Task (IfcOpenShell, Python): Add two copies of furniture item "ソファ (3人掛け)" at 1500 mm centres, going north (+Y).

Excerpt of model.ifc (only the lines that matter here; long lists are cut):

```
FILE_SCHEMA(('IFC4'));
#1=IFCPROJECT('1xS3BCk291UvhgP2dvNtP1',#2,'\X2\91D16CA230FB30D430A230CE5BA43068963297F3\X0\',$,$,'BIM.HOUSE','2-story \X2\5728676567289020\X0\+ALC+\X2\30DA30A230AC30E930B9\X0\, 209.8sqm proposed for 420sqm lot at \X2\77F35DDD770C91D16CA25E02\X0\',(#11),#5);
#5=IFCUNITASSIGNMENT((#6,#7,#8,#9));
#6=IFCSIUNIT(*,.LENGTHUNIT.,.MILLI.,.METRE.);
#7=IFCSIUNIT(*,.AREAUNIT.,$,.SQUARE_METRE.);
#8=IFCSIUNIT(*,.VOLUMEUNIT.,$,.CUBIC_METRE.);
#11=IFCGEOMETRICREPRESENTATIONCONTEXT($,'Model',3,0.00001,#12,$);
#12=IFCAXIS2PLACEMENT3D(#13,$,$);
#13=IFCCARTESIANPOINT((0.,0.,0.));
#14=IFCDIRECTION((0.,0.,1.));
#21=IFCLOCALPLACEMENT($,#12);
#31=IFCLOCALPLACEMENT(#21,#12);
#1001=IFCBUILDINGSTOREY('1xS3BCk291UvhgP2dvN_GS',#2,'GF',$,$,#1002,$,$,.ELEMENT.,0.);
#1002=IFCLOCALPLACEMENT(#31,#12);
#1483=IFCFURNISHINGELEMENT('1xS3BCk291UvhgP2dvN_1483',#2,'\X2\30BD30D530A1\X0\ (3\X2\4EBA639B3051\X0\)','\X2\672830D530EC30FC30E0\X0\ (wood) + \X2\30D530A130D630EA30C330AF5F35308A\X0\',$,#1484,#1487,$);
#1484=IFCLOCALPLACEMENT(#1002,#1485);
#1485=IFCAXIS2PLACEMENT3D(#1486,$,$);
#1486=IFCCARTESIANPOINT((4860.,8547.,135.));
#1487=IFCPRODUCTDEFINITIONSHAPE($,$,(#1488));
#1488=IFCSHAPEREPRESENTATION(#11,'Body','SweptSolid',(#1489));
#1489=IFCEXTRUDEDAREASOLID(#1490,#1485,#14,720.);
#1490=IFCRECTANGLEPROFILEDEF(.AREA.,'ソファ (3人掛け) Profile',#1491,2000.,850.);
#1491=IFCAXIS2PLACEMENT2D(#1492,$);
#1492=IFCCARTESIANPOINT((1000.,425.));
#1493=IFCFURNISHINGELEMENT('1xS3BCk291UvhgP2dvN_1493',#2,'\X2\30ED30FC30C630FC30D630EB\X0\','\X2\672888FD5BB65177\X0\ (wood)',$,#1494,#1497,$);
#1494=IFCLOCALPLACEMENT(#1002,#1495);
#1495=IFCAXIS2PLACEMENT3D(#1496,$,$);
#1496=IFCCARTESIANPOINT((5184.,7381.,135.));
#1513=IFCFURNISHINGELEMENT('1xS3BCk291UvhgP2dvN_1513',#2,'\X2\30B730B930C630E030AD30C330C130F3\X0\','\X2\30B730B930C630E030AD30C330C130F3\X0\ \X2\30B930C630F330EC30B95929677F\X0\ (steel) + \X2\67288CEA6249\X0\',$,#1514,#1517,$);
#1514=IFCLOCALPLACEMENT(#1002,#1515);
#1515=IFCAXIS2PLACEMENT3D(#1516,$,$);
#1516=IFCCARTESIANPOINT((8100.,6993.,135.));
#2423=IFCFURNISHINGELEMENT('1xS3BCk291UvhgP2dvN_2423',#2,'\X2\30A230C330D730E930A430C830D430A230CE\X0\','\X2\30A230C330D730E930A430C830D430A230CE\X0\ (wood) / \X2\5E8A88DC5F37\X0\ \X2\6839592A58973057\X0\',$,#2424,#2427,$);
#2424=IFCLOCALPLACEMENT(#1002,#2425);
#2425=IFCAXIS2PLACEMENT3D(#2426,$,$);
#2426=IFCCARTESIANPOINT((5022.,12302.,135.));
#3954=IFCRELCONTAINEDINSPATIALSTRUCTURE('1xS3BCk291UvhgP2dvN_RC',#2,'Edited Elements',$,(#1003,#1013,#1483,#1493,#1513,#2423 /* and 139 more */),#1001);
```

```python
import numpy as np
import ifcopenshell
import ifcopenshell.api.geometry
import ifcopenshell.api.root
import ifcopenshell.util.element
import ifcopenshell.util.placement
import ifcopenshell.util.unit

model = ifcopenshell.open("model.ifc")
unit_scale = ifcopenshell.util.unit.calculate_unit_scale(model)


def reuse_history(source, copy):
    """copy_class also copies each property set's owner history, people and application; keep the originals."""
    for rel in copy.IsDefinedBy:
        if rel.is_a("IfcRelDefinesByProperties") and (history := rel.RelatingPropertyDefinition.OwnerHistory):
            rel.RelatingPropertyDefinition.OwnerHistory = source.OwnerHistory
            ifcopenshell.util.element.remove_deep2(model, history)


source = model.by_guid("1xS3BCk291UvhgP2dvN_1483")
base = ifcopenshell.util.placement.get_local_placement(source.ObjectPlacement)
step = np.array([0.0, 1.0, 0.0]) * 1.5 / unit_scale

for i in range(1, 3):
    copy = ifcopenshell.api.root.copy_class(model, product=source)
    copy.Representation = ifcopenshell.util.element.copy_deep(
        model, source.Representation, exclude=["IfcGeometricRepresentationContext", "IfcRepresentationMap"]
    )
    reuse_history(source, copy)
    matrix = base.copy()
    matrix[:3, 3] += i * step
    print("added at", matrix[:3, 3].round(3) + 0.0)
    ifcopenshell.api.geometry.edit_object_placement(model, product=copy, matrix=matrix, is_si=False)

model.write("model_updated.ifc")
```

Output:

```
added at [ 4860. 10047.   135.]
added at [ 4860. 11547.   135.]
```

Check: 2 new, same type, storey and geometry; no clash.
